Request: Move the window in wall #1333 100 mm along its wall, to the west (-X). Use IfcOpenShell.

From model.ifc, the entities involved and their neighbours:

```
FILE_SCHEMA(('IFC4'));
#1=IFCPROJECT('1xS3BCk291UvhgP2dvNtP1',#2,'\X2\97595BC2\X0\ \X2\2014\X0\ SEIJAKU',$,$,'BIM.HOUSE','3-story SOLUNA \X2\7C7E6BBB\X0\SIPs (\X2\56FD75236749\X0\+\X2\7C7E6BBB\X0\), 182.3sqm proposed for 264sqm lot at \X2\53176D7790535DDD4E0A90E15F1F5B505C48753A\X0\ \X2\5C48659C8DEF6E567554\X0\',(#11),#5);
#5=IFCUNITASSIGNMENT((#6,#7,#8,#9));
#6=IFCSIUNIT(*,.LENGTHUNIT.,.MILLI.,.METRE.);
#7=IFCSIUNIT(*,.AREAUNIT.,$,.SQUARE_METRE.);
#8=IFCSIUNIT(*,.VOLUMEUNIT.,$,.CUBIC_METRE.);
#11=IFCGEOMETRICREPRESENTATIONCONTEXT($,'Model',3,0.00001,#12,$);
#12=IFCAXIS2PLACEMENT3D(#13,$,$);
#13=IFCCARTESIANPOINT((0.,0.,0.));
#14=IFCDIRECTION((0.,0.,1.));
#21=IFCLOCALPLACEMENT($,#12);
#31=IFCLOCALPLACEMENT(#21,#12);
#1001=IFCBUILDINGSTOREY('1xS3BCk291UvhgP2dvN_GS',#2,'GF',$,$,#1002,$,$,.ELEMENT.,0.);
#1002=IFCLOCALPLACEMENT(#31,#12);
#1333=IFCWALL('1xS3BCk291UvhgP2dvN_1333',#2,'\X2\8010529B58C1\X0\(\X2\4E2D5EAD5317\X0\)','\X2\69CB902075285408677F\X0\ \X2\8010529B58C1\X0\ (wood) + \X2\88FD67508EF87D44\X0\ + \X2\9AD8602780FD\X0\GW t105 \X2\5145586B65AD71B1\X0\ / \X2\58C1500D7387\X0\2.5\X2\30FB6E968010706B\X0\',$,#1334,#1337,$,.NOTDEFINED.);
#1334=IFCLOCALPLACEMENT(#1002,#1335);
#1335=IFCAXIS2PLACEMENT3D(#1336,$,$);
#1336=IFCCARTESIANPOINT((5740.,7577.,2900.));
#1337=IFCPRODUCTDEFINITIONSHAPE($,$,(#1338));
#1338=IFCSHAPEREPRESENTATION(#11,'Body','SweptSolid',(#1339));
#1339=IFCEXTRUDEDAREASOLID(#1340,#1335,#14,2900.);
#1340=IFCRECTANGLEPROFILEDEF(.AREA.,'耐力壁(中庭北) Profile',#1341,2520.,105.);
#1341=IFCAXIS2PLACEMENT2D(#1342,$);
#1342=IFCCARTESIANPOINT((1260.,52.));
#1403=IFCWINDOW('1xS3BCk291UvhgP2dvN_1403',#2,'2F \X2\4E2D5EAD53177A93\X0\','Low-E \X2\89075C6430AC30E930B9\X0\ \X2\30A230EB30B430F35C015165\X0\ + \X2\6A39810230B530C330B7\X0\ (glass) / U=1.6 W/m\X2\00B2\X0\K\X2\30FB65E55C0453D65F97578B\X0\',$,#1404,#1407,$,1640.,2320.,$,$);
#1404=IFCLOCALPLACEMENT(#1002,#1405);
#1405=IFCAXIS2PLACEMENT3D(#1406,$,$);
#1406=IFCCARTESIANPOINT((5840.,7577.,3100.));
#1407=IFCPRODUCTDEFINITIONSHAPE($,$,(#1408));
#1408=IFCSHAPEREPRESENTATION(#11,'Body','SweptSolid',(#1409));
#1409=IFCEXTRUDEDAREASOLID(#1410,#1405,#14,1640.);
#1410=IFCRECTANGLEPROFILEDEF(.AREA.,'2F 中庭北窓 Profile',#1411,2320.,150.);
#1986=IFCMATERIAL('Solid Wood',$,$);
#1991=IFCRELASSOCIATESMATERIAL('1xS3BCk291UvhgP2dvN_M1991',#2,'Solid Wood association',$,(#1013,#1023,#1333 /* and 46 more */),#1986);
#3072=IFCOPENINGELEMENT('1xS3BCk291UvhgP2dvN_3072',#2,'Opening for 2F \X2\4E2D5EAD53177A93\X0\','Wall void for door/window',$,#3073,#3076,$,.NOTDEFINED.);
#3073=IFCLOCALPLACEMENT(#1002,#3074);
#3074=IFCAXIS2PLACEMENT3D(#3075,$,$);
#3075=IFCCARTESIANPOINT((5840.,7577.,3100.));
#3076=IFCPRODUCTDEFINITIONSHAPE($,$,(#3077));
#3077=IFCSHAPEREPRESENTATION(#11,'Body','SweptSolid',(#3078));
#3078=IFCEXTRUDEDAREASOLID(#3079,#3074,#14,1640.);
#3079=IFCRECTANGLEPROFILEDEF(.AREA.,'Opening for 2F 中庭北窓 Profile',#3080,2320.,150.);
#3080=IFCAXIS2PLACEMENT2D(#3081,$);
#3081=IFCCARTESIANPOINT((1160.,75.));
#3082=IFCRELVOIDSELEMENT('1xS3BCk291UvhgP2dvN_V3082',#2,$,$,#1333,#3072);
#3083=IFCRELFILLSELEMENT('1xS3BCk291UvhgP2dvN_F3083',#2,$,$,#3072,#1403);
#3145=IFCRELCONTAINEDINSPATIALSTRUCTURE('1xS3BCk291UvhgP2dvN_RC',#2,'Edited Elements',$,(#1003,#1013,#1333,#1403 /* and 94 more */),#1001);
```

```python
import ifcopenshell
import ifcopenshell.api.geometry
import ifcopenshell.util.placement

model = ifcopenshell.open("model.ifc")

window = model.by_guid("1xS3BCk291UvhgP2dvN_1403")
opening = window.FillsVoids[0].RelatingOpeningElement
wall = opening.VoidsElements[0].RelatingBuildingElement

wall_matrix = ifcopenshell.util.placement.get_local_placement(wall.ObjectPlacement)
shift = wall_matrix[:3, 0] * -100.0
before = ifcopenshell.util.placement.get_local_placement(window.ObjectPlacement)[:3, 3].copy()

# The window is not placed relative to its opening, so move both.
for product in (opening, window):
    matrix = ifcopenshell.util.placement.get_local_placement(product.ObjectPlacement)
    matrix[:3, 3] += shift
    ifcopenshell.api.geometry.edit_object_placement(model, product=product, matrix=matrix, is_si=False)

after = ifcopenshell.util.placement.get_local_placement(window.ObjectPlacement)[:3, 3]
print("window moved by", (after - before).round(3) + 0.0)

model.write("model_v2.ifc")
```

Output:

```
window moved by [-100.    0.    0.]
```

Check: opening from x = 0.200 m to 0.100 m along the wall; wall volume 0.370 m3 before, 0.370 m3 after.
